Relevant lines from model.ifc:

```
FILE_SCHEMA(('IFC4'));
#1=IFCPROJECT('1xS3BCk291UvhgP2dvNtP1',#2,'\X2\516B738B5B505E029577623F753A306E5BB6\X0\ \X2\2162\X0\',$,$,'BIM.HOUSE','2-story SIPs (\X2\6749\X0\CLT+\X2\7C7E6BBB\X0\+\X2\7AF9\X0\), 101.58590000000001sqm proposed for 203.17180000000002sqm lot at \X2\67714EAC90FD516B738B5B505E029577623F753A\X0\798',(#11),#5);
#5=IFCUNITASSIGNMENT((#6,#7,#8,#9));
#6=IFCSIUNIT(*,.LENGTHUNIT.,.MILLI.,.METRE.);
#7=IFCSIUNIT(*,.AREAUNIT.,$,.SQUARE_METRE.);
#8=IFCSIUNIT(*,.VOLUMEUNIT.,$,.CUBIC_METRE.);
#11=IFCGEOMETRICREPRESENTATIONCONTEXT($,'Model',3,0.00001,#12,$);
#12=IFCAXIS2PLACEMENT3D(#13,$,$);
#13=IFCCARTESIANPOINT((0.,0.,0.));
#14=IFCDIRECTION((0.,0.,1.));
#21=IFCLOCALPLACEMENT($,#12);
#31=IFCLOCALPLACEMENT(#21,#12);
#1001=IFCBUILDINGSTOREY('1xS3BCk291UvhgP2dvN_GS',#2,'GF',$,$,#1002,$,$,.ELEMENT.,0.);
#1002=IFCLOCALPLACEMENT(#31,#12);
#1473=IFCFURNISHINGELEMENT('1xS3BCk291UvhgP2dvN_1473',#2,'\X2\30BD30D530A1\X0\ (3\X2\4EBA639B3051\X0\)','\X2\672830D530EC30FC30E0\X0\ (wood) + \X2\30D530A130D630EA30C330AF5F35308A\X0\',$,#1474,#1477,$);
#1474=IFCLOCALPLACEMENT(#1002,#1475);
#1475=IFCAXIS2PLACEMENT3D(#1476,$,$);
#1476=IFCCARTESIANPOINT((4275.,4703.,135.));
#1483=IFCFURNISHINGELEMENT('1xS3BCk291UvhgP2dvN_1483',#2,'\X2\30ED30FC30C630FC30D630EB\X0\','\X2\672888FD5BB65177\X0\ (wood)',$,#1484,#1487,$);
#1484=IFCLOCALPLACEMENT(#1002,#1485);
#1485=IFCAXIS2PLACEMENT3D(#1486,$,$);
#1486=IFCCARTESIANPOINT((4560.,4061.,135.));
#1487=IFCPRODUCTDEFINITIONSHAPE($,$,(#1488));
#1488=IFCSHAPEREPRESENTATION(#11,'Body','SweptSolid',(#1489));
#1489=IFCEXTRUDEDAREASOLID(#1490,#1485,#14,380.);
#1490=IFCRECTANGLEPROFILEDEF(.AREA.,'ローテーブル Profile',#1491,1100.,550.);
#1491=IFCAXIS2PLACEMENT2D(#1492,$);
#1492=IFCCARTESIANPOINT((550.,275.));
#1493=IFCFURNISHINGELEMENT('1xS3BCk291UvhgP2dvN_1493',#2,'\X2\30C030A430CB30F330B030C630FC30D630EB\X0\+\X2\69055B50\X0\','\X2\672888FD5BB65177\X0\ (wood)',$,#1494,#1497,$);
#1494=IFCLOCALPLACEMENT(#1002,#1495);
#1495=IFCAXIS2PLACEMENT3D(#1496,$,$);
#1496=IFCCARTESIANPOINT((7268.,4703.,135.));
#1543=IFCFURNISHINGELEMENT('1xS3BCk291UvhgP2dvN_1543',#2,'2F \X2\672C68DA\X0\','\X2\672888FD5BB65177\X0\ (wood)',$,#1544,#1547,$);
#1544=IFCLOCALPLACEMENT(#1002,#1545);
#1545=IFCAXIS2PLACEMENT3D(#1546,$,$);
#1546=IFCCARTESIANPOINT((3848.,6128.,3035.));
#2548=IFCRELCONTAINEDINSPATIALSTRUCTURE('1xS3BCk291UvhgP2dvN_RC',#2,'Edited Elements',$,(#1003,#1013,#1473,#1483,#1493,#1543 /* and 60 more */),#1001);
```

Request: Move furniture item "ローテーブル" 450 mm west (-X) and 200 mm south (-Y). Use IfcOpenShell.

```python
import ifcopenshell
import ifcopenshell.api.geometry
import ifcopenshell.util.placement
import ifcopenshell.util.unit

model = ifcopenshell.open("model.ifc")
unit_scale = ifcopenshell.util.unit.calculate_unit_scale(model)

item = model.by_guid("1xS3BCk291UvhgP2dvN_1483")
matrix = ifcopenshell.util.placement.get_local_placement(item.ObjectPlacement)
matrix[0, 3] -= 0.45 / unit_scale
matrix[1, 3] -= 0.2 / unit_scale
ifcopenshell.api.geometry.edit_object_placement(model, product=item, matrix=matrix, is_si=False)

print(ifcopenshell.util.placement.get_local_placement(item.ObjectPlacement).round(3) + 0.0)

model.write("model_v2.ifc")
```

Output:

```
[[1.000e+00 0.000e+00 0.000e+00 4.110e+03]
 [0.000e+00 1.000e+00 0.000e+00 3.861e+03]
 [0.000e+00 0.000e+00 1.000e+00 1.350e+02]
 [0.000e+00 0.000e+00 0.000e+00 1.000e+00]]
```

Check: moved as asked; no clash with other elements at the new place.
